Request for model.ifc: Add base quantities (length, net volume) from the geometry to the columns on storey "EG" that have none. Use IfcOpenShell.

First a look at what the model holds.

```python
import ifcopenshell
import ifcopenshell.util.element
import ifcopenshell.util.unit

model = ifcopenshell.open("model.ifc")
print(model.schema)
for unit_type in ("LENGTHUNIT", "AREAUNIT", "VOLUMEUNIT"):
    print(unit_type, ifcopenshell.util.unit.calculate_unit_scale(model, unit_type))
storey = next(s for s in model.by_type("IfcBuildingStorey") if s.Name == "EG")
columns = [e for e in ifcopenshell.util.element.get_decomposition(storey) if e.is_a("IfcColumn")]
for e in sorted(columns, key=lambda e: e.id()):
    print(e.id(), e.is_a(), e.Name, list(ifcopenshell.util.element.get_psets(e, qtos_only=True)), sep=" | ")
```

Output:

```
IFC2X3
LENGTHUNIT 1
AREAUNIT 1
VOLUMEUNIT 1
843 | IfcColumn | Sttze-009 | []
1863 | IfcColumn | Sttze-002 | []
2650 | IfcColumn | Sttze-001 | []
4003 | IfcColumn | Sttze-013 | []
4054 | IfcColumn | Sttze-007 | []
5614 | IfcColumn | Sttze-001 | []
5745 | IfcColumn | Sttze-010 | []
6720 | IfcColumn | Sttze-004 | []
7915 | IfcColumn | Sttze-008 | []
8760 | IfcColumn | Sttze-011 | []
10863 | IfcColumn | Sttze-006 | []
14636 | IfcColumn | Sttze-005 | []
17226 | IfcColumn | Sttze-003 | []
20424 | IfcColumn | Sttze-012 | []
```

```python
import ifcopenshell
import ifcopenshell.api.pset
import ifcopenshell.geom
import ifcopenshell.util.element
import ifcopenshell.util.shape
import ifcopenshell.util.unit

model = ifcopenshell.open("model.ifc")
unit_scale = ifcopenshell.util.unit.calculate_unit_scale(model)
volume_scale = ifcopenshell.util.unit.calculate_unit_scale(model, "VOLUMEUNIT")
settings = ifcopenshell.geom.settings()

storey = next(s for s in model.by_type("IfcBuildingStorey") if s.Name == "EG")
columns = [e for e in ifcopenshell.util.element.get_decomposition(storey) if e.is_a("IfcColumn")]

for e in sorted(columns, key=lambda e: e.id()):
    if ifcopenshell.util.element.get_psets(e, qtos_only=True, should_inherit=False):
        continue
    # Geometry comes back in metres, in the element's own axes.
    shape = ifcopenshell.geom.create_shape(settings, e)
    values = {
        "Length": ifcopenshell.util.shape.get_z(shape.geometry) / unit_scale,
        "NetVolume": ifcopenshell.util.shape.get_volume(shape.geometry) / volume_scale,
    }
    qto = ifcopenshell.api.pset.add_qto(model, product=e, name="BaseQuantities")
    ifcopenshell.api.pset.edit_qto(model, qto=qto, properties=values)
    print(e.id(), {k: round(v, 3) for k, v in values.items()})

model.write("model_v2.ifc")
```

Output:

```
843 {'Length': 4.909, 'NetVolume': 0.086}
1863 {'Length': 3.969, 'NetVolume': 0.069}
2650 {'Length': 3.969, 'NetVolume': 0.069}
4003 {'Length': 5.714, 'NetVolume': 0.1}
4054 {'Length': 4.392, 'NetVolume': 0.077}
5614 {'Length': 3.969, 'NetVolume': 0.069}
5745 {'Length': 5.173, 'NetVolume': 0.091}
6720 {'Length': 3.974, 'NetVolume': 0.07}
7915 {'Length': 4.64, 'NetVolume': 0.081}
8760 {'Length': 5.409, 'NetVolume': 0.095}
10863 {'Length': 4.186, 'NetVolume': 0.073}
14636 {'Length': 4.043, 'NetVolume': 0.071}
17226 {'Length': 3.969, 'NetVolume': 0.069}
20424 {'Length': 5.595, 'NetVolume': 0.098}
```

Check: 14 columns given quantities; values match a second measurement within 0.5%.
